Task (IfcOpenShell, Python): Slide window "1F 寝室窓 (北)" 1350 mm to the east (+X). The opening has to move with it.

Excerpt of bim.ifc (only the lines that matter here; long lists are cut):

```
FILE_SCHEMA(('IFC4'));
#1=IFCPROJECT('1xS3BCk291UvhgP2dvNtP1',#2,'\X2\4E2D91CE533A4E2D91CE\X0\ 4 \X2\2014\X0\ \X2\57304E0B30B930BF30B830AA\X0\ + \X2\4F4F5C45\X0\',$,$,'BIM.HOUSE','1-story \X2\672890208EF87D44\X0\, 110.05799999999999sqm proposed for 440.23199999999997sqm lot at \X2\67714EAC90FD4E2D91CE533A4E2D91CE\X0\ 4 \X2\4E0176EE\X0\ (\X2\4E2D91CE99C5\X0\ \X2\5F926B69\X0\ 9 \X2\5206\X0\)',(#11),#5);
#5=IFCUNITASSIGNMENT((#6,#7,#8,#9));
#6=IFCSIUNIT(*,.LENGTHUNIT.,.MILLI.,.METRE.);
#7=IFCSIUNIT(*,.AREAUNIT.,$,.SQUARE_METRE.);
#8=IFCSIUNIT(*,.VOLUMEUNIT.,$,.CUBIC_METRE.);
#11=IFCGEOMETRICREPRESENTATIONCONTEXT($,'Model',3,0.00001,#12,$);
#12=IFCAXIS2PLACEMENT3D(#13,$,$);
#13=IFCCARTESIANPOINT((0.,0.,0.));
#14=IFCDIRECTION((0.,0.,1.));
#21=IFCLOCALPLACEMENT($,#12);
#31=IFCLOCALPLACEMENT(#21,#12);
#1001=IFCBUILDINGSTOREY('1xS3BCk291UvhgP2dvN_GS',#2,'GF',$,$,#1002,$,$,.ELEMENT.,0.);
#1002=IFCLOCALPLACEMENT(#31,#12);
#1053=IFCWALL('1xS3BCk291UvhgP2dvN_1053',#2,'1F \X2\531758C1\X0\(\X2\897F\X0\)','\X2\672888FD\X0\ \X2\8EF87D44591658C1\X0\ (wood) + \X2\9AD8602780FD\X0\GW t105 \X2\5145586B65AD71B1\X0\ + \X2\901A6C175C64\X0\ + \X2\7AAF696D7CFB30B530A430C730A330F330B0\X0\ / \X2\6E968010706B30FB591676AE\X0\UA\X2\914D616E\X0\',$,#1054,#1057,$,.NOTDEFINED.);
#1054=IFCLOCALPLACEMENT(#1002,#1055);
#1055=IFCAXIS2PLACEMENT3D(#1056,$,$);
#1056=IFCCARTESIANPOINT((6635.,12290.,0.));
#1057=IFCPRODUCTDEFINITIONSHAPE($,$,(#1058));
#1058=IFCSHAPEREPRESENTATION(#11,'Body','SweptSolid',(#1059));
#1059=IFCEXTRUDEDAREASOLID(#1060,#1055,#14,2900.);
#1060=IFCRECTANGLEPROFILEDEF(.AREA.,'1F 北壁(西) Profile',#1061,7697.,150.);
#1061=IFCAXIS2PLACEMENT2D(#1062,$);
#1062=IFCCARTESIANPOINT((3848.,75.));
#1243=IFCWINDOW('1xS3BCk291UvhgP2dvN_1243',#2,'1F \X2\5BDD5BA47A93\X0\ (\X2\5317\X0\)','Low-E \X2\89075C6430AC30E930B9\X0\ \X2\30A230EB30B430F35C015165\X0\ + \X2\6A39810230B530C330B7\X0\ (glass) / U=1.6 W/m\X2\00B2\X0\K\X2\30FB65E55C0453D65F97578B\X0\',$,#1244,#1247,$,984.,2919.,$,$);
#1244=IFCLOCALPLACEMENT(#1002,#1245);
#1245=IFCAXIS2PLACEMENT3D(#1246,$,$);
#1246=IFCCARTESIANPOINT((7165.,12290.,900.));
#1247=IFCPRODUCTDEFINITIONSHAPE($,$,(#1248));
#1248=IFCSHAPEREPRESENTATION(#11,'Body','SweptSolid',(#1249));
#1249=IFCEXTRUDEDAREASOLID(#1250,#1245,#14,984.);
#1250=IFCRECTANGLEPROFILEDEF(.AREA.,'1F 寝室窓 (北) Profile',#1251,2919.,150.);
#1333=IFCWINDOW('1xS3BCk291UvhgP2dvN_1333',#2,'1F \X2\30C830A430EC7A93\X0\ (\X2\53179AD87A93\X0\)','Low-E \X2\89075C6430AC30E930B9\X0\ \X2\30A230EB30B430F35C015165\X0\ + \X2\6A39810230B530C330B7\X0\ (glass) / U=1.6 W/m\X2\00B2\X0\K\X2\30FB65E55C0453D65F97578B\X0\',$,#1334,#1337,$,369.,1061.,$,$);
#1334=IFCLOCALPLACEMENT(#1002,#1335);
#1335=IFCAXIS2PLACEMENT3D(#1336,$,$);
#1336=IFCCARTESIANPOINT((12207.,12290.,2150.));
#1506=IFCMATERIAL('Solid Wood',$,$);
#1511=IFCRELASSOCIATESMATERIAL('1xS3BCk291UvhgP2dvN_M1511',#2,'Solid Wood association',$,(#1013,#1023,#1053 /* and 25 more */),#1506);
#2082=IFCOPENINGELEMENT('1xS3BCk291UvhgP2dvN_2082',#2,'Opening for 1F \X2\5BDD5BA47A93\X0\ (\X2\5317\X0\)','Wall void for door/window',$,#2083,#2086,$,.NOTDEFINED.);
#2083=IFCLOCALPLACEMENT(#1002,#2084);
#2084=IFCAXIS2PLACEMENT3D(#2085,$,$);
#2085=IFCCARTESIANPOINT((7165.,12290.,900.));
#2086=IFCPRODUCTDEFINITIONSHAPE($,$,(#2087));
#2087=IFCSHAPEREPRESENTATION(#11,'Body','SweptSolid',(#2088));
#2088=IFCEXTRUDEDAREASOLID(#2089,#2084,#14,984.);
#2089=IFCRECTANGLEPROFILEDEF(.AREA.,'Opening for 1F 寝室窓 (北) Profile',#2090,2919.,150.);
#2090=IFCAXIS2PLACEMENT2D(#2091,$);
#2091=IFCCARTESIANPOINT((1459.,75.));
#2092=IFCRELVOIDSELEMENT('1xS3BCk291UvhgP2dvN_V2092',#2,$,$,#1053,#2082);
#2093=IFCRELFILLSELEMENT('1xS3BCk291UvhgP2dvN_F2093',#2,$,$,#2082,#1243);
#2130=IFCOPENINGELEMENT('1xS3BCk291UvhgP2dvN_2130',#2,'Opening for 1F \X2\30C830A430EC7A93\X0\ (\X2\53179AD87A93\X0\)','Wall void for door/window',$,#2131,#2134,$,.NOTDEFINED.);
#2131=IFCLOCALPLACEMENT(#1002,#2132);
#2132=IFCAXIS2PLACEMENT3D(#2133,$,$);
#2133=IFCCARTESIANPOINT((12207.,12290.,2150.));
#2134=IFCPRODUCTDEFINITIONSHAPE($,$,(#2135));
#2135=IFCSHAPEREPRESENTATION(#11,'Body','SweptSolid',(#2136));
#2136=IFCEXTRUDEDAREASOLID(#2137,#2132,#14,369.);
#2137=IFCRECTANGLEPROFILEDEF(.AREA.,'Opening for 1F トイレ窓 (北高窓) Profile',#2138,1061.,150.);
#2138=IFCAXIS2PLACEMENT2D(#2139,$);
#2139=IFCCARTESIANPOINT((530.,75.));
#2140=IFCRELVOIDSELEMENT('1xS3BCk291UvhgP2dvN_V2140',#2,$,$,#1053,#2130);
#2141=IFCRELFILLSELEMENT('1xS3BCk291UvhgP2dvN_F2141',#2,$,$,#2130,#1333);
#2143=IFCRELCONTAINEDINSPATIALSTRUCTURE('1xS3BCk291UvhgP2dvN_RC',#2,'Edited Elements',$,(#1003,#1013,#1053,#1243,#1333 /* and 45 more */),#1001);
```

```python
import ifcopenshell
import ifcopenshell.api.geometry
import ifcopenshell.util.placement
import ifcopenshell.util.unit

model = ifcopenshell.open("bim.ifc")
unit_scale = ifcopenshell.util.unit.calculate_unit_scale(model)

window = model.by_guid("1xS3BCk291UvhgP2dvN_1243")
opening = window.FillsVoids[0].RelatingOpeningElement
wall = opening.VoidsElements[0].RelatingBuildingElement

wall_matrix = ifcopenshell.util.placement.get_local_placement(wall.ObjectPlacement)
shift = wall_matrix[:3, 0] * 1.35 / unit_scale
before = ifcopenshell.util.placement.get_local_placement(window.ObjectPlacement)[:3, 3].copy()

# The window is not placed relative to its opening, so move both.
for product in (opening, window):
    matrix = ifcopenshell.util.placement.get_local_placement(product.ObjectPlacement)
    matrix[:3, 3] += shift
    ifcopenshell.api.geometry.edit_object_placement(model, product=product, matrix=matrix, is_si=False)

after = ifcopenshell.util.placement.get_local_placement(window.ObjectPlacement)[:3, 3]
print("window moved by", (after - before).round(3) + 0.0)

model.write("bim_updated.ifc")
```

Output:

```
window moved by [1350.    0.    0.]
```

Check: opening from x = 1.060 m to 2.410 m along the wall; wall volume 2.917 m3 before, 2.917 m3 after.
